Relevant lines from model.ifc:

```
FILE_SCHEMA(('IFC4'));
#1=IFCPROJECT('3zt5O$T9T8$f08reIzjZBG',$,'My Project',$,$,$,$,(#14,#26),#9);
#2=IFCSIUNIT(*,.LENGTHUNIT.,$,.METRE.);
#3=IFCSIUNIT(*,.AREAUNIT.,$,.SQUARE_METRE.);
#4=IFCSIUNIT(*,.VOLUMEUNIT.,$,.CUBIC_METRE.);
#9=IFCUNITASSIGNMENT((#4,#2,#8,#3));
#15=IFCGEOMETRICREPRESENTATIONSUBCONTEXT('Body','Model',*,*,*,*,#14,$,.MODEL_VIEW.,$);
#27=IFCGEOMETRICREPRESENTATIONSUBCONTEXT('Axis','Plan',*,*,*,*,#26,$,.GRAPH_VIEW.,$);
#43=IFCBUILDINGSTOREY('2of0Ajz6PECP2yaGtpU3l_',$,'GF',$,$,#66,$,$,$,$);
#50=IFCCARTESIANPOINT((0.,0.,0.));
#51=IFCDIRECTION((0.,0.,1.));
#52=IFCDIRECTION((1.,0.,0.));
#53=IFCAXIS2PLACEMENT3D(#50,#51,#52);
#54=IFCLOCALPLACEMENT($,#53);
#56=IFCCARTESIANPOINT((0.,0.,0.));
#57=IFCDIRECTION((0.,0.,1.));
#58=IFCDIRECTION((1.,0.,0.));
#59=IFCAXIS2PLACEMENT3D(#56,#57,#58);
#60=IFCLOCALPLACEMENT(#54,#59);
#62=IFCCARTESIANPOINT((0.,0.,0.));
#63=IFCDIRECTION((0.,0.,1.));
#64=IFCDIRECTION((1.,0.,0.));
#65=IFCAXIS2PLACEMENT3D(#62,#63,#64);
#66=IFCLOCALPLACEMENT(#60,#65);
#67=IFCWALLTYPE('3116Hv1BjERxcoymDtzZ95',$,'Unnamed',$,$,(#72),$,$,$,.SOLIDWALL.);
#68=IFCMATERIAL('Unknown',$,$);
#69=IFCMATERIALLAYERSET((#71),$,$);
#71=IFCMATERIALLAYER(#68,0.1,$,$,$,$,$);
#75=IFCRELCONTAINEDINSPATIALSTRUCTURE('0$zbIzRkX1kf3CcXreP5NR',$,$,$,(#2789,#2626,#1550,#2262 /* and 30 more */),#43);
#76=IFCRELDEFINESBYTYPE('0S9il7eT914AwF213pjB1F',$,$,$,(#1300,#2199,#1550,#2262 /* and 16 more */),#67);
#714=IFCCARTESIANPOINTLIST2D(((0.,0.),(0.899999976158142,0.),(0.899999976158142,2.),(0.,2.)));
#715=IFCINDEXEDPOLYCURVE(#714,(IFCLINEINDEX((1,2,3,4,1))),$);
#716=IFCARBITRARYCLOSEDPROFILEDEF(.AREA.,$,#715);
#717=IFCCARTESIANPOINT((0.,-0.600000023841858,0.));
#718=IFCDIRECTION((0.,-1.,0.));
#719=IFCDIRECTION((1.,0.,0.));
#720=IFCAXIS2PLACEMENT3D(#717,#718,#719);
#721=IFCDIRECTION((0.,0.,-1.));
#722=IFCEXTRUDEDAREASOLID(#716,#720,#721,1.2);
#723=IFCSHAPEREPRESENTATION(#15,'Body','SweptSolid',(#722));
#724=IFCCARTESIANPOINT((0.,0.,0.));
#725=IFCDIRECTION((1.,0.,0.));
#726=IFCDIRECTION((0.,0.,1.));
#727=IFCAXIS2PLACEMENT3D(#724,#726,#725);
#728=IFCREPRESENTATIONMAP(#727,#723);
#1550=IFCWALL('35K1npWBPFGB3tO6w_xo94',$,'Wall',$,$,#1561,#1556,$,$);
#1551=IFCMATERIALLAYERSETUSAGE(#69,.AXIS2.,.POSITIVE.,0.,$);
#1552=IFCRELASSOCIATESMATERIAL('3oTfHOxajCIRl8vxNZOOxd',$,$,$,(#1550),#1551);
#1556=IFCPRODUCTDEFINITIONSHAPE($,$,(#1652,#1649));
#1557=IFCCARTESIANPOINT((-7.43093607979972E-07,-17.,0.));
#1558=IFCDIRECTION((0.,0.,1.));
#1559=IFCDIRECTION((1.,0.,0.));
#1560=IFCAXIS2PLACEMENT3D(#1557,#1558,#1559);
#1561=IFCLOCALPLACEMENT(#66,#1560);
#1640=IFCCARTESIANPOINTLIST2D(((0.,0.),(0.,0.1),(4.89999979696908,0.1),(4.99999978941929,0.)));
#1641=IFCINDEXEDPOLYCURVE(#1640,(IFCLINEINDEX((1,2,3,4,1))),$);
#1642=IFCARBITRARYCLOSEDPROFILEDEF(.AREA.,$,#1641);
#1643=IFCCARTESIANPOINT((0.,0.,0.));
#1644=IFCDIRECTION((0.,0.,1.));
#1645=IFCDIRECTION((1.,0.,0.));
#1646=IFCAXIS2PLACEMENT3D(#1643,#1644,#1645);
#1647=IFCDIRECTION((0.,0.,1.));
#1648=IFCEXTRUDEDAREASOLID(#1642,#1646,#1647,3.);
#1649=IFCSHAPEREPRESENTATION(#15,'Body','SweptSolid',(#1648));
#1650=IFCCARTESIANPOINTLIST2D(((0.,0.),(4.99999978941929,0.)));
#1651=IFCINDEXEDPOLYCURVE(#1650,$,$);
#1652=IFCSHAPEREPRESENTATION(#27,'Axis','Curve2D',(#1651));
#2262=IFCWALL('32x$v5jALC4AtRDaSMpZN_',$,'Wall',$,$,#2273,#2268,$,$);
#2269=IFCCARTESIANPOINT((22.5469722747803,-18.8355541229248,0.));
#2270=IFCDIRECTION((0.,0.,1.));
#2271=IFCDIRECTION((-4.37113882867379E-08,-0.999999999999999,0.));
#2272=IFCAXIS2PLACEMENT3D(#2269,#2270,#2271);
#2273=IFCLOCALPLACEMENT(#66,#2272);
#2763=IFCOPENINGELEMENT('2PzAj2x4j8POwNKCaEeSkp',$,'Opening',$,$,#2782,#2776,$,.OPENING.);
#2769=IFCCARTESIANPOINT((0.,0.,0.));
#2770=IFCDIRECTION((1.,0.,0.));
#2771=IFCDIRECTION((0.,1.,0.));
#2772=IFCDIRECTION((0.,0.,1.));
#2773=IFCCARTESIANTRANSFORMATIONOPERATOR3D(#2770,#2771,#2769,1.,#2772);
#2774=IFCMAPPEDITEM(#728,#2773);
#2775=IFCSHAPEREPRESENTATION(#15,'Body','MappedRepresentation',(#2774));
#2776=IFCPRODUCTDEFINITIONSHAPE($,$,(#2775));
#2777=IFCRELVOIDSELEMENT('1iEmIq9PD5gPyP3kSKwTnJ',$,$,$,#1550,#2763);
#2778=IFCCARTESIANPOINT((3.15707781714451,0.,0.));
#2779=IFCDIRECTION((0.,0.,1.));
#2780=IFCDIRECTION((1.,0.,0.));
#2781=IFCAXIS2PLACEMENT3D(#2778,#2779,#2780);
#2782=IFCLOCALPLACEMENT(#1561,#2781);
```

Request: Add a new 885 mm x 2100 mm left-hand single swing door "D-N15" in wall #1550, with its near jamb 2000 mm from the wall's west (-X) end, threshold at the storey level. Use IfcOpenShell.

```python
import numpy as np
import ifcopenshell
import ifcopenshell.api.feature
import ifcopenshell.api.geometry
import ifcopenshell.api.root
import ifcopenshell.api.spatial
import ifcopenshell.geom
import ifcopenshell.util.element
import ifcopenshell.util.placement
import ifcopenshell.util.representation
import ifcopenshell.util.shape
import ifcopenshell.util.unit

model = ifcopenshell.open("model.ifc")
unit_scale = ifcopenshell.util.unit.calculate_unit_scale(model)
settings = ifcopenshell.geom.settings()


def volume(element):
    """Net volume in cubic metres, openings subtracted."""
    shape = ifcopenshell.geom.create_shape(settings, element)
    return ifcopenshell.util.shape.get_volume(shape.geometry)


wall = model.by_guid("35K1npWBPFGB3tO6w_xo94")
storey = ifcopenshell.util.element.get_container(wall, ifc_class="IfcBuildingStorey")
context = ifcopenshell.util.representation.get_context(model, "Model", "Body", "MODEL_VIEW")
before = volume(wall)

width, height, from_end, sill = 0.885, 2.1, 2, 0.0  # metres

# The wall runs along its own X axis, and the end named is its -X end.
wall_shape = ifcopenshell.geom.create_shape(settings, wall)
x, y, z = ifcopenshell.util.shape.get_vertices(wall_shape.geometry).T
start = x.min() + from_end
face, thickness = float(y.min()), float(y.max() - y.min())
wall_matrix = ifcopenshell.util.placement.get_local_placement(wall.ObjectPlacement)
level = ifcopenshell.util.placement.get_local_placement(storey.ObjectPlacement)[2, 3]


def in_wall(x, y):
    """Placement at x, y metres in the wall's axes, at sill height."""
    matrix = wall_matrix.copy()
    matrix[:, 3] = wall_matrix @ np.array([x / unit_scale, y / unit_scale, 0.0, 1.0])
    matrix[2, 3] = level + sill / unit_scale
    return matrix


# Opening: a box that overshoots both wall faces by 50 mm.
opening = ifcopenshell.api.root.create_entity(model, ifc_class="IfcOpeningElement", predefined_type="OPENING")
box = ifcopenshell.api.geometry.add_wall_representation(
    model, context=context, length=width, height=height, thickness=thickness + 0.1
)
ifcopenshell.api.geometry.assign_representation(model, product=opening, representation=box)
ifcopenshell.api.geometry.edit_object_placement(model, product=opening, matrix=in_wall(start, face - 0.05), is_si=False)
ifcopenshell.api.feature.add_feature(model, feature=opening, element=wall)

door = ifcopenshell.api.root.create_entity(model, ifc_class="IfcDoor", name="D-N15", predefined_type="DOOR")
door.OverallWidth, door.OverallHeight = width / unit_scale, height / unit_scale
door.OperationType = "SINGLE_SWING_LEFT"
body = ifcopenshell.api.geometry.add_door_representation(
    model,
    context=context,
    overall_width=door.OverallWidth,
    overall_height=door.OverallHeight,
    operation_type="SINGLE_SWING_LEFT",
    lining_properties={"LiningDepth": thickness / unit_scale, "ThresholdDepth": thickness / unit_scale},
)
ifcopenshell.api.geometry.assign_representation(model, product=door, representation=body)
ifcopenshell.api.spatial.assign_container(model, products=[door], relating_structure=storey)
ifcopenshell.api.feature.add_filling(model, opening=opening, element=door)

# The lining spans the wall, so the door starts at the wall face.
ifcopenshell.api.geometry.edit_object_placement(model, product=door, matrix=in_wall(start, face), is_si=False)

after = volume(wall)

print(f"wall volume {before:.3f} -> {after:.3f} m3")

model.write("model_updated.ifc")
```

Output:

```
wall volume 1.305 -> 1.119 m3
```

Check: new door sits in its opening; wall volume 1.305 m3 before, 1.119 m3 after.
